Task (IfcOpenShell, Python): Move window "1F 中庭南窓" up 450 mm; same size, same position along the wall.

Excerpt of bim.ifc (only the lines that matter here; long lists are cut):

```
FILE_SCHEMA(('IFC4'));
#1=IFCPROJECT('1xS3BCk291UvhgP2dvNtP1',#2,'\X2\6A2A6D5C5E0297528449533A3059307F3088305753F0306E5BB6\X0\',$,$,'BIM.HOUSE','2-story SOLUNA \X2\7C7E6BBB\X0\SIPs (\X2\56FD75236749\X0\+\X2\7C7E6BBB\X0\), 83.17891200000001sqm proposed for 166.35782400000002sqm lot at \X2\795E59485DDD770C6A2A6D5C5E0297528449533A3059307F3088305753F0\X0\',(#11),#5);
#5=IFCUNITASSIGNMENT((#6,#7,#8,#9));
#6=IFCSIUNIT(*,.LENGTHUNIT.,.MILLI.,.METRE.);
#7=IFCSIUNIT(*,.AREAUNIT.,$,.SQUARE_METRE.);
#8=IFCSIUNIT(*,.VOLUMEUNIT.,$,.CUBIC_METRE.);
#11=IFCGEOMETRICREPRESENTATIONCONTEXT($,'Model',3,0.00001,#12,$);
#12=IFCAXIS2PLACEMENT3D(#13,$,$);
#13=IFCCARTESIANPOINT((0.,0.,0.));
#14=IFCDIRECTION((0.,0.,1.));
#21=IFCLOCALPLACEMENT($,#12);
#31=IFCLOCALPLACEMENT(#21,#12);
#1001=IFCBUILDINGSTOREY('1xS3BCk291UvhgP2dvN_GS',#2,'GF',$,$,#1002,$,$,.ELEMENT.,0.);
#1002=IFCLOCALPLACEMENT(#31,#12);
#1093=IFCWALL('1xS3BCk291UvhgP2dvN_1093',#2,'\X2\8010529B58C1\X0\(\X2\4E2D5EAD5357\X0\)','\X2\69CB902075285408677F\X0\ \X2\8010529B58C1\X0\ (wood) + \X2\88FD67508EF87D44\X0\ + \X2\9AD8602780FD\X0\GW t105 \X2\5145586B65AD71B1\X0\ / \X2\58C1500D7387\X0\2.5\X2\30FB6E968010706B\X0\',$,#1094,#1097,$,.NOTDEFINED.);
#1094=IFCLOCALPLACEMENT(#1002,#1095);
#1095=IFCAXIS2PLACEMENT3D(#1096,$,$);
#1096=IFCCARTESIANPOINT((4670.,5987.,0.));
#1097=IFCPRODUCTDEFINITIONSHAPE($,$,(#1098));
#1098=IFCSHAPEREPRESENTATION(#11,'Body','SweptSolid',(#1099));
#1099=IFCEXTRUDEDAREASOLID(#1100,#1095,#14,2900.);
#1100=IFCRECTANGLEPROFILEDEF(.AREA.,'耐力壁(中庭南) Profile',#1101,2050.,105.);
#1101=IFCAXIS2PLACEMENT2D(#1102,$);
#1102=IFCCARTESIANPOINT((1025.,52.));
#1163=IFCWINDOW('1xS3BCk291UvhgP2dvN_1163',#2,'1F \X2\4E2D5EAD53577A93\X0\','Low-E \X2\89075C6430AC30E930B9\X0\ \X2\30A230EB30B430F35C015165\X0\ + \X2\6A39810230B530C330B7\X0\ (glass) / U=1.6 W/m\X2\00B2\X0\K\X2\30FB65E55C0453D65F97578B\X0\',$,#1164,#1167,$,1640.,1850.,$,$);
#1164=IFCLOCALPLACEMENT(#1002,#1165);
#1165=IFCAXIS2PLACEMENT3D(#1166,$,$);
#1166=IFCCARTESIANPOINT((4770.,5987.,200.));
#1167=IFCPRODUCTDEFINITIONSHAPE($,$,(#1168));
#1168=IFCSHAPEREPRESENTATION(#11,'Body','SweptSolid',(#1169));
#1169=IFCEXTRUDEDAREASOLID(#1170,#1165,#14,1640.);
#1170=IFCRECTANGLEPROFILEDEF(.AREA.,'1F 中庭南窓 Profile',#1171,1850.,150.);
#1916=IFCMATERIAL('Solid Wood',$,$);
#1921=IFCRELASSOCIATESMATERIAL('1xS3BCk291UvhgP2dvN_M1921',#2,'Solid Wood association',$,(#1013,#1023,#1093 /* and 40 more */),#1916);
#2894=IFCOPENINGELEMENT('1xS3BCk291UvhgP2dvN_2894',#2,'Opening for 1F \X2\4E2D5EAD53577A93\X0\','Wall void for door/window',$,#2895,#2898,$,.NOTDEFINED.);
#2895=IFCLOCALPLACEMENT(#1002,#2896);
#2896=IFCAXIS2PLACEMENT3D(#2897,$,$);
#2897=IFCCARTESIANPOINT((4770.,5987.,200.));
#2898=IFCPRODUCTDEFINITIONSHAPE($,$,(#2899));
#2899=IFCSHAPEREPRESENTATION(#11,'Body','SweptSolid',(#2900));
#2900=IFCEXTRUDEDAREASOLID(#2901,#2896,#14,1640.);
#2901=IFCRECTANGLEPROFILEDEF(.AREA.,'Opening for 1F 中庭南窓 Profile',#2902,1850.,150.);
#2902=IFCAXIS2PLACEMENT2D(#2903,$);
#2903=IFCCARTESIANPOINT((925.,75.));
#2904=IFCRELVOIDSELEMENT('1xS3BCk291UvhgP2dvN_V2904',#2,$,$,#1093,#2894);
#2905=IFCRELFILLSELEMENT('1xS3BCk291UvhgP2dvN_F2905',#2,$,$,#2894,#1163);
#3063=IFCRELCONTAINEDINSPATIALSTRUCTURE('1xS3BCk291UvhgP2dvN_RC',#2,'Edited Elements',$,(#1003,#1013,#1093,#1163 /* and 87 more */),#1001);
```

```python
import numpy as np
import ifcopenshell
import ifcopenshell.api.geometry
import ifcopenshell.util.placement
import ifcopenshell.util.unit

model = ifcopenshell.open("bim.ifc")
unit_scale = ifcopenshell.util.unit.calculate_unit_scale(model)

window = model.by_guid("1xS3BCk291UvhgP2dvN_1163")
opening = window.FillsVoids[0].RelatingOpeningElement
dz = 0.45 / unit_scale

shift = np.array([0.0, 0.0, dz])
# The window is not placed relative to its opening, so move both.
for product in (opening, window):
    matrix = ifcopenshell.util.placement.get_local_placement(product.ObjectPlacement)
    matrix[:3, 3] += shift
    ifcopenshell.api.geometry.edit_object_placement(model, product=product, matrix=matrix, is_si=False)

print(f"moved by {dz * unit_scale:+.3f} m")

model.write("bim_rev.ifc")
```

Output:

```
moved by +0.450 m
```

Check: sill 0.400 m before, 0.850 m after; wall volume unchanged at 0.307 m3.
